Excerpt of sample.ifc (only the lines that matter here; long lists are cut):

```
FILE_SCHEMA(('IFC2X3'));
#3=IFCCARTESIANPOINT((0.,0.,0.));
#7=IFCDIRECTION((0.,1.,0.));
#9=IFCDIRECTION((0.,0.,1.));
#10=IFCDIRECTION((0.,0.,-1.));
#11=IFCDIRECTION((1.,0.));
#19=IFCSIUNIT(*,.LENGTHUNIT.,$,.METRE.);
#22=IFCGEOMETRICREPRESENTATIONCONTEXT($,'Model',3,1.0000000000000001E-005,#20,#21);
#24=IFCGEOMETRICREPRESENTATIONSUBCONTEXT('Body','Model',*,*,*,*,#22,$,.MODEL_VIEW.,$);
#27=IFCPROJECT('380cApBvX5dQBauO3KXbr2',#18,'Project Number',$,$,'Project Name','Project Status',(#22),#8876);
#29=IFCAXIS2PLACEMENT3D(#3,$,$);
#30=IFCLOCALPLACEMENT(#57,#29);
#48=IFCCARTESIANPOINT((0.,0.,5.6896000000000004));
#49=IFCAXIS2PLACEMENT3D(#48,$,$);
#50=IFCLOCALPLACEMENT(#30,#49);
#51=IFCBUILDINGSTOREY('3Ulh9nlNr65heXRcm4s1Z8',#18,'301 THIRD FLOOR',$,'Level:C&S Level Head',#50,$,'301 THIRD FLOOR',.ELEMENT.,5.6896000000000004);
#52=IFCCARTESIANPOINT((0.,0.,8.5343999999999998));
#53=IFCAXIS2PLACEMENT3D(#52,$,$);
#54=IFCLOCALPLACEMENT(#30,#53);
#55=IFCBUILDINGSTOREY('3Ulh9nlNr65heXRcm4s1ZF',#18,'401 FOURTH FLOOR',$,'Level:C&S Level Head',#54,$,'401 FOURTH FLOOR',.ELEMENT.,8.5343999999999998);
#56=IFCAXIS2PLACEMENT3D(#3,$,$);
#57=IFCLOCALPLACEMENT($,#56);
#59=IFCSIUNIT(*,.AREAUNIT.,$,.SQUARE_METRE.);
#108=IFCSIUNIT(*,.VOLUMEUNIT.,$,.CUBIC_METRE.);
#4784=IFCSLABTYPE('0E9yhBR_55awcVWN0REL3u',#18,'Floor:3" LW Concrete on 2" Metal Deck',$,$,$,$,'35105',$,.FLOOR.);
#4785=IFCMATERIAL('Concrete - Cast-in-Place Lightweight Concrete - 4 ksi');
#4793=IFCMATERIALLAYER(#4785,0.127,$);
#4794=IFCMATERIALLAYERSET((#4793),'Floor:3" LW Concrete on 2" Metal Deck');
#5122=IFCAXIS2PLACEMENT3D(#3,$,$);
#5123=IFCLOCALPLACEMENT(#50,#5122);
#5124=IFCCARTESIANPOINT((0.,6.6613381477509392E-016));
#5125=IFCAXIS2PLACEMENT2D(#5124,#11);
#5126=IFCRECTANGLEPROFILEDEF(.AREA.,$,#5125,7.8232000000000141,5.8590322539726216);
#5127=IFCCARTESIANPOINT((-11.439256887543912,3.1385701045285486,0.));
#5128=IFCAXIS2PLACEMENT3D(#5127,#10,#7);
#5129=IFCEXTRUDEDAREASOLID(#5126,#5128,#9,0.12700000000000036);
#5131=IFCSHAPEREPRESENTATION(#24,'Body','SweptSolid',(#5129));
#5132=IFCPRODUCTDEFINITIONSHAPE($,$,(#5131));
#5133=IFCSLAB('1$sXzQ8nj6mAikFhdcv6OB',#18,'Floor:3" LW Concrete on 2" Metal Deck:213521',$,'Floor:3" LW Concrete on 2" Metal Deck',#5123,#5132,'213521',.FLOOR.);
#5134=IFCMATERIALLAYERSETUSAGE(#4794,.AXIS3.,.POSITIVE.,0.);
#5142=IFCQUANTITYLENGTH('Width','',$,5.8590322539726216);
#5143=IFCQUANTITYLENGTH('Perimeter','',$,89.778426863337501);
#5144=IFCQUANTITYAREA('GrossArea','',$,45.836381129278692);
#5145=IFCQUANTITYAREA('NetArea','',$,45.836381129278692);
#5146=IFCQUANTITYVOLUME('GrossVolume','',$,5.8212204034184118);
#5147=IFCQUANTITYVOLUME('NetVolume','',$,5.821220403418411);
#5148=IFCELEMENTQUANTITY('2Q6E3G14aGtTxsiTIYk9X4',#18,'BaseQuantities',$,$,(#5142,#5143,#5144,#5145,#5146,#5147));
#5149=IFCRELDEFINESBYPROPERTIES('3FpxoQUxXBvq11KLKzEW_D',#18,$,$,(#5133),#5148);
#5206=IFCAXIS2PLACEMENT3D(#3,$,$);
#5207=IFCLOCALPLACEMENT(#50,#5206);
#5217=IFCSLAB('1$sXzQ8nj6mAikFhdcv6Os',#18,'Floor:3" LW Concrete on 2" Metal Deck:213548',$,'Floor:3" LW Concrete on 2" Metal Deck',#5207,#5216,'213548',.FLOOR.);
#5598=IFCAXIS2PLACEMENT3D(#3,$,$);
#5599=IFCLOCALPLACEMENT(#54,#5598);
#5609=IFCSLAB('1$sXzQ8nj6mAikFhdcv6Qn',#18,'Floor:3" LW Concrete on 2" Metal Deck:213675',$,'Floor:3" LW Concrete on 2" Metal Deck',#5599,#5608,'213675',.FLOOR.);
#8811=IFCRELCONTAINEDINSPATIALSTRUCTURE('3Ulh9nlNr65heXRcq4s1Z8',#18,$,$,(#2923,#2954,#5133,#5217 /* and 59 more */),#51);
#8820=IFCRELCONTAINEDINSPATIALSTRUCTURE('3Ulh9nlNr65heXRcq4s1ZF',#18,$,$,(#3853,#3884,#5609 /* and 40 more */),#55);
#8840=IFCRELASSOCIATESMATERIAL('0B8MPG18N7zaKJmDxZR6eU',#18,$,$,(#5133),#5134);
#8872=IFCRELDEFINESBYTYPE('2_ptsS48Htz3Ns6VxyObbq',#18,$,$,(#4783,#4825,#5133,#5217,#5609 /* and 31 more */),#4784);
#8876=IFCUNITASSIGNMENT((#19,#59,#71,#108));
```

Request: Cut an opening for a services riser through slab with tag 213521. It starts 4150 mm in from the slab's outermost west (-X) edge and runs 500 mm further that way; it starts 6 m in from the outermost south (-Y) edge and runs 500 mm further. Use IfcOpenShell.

```python
import numpy as np
import ifcopenshell
import ifcopenshell.api.feature
import ifcopenshell.api.geometry
import ifcopenshell.api.pset
import ifcopenshell.api.root
import ifcopenshell.geom
import ifcopenshell.util.element
import ifcopenshell.util.placement
import ifcopenshell.util.representation
import ifcopenshell.util.shape
import ifcopenshell.util.unit

model = ifcopenshell.open("sample.ifc")
unit_scale = ifcopenshell.util.unit.calculate_unit_scale(model)
area_scale = ifcopenshell.util.unit.calculate_unit_scale(model, "AREAUNIT")
volume_scale = ifcopenshell.util.unit.calculate_unit_scale(model, "VOLUMEUNIT")
settings = ifcopenshell.geom.settings()


def volume(element):
    """Net volume in cubic metres, openings subtracted."""
    shape = ifcopenshell.geom.create_shape(settings, element)
    return ifcopenshell.util.shape.get_volume(shape.geometry)


slab = model.by_guid("1$sXzQ8nj6mAikFhdcv6OB")
before = volume(slab)

# Extent in the slab's own axes, in metres. The edges named are its -X and -Y sides.
slab_shape = ifcopenshell.geom.create_shape(settings, slab)
vertices = ifcopenshell.util.shape.get_vertices(slab_shape.geometry)
x_min, y_min, bottom = vertices.min(axis=0)
top = vertices[:, 2].max()

opening = ifcopenshell.api.root.create_entity(model, ifc_class="IfcOpeningElement", name="Services riser opening")
context = ifcopenshell.util.representation.get_context(model, "Model", "Body", "MODEL_VIEW")
width, depth = 0.5, 0.5
outline = [(0.0, 0.0), (width, 0.0), (width, depth), (0.0, depth), (0.0, 0.0)]
# Overshoot both faces by 50 mm so the cut is clean.
shape = ifcopenshell.api.geometry.add_slab_representation(
    model, context=context, depth=top - bottom + 0.1, polyline=outline
)
ifcopenshell.api.geometry.assign_representation(model, product=opening, representation=shape)

matrix = ifcopenshell.util.placement.get_local_placement(slab.ObjectPlacement)
matrix[:, 3] = matrix @ np.append(np.array([x_min + 4.15, y_min + 6, bottom - 0.05]) / unit_scale, 1.0)
ifcopenshell.api.geometry.edit_object_placement(model, product=opening, matrix=matrix, is_si=False)
ifcopenshell.api.feature.add_feature(model, feature=opening, element=slab)

after = volume(slab)

# Update the slab's stored quantities.
qto = model.by_id(ifcopenshell.util.element.get_pset(slab, "BaseQuantities", should_inherit=False)["id"])
ifcopenshell.api.pset.edit_qto(model, qto=qto, properties={
    "NetArea": after / (top - bottom) / area_scale,
    "NetVolume": after / volume_scale,
})

print(f"slab volume {before:.3f} -> {after:.3f} m3")

model.write("sample_edited.ifc")
```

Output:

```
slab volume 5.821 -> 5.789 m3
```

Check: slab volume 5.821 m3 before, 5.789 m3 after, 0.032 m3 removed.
